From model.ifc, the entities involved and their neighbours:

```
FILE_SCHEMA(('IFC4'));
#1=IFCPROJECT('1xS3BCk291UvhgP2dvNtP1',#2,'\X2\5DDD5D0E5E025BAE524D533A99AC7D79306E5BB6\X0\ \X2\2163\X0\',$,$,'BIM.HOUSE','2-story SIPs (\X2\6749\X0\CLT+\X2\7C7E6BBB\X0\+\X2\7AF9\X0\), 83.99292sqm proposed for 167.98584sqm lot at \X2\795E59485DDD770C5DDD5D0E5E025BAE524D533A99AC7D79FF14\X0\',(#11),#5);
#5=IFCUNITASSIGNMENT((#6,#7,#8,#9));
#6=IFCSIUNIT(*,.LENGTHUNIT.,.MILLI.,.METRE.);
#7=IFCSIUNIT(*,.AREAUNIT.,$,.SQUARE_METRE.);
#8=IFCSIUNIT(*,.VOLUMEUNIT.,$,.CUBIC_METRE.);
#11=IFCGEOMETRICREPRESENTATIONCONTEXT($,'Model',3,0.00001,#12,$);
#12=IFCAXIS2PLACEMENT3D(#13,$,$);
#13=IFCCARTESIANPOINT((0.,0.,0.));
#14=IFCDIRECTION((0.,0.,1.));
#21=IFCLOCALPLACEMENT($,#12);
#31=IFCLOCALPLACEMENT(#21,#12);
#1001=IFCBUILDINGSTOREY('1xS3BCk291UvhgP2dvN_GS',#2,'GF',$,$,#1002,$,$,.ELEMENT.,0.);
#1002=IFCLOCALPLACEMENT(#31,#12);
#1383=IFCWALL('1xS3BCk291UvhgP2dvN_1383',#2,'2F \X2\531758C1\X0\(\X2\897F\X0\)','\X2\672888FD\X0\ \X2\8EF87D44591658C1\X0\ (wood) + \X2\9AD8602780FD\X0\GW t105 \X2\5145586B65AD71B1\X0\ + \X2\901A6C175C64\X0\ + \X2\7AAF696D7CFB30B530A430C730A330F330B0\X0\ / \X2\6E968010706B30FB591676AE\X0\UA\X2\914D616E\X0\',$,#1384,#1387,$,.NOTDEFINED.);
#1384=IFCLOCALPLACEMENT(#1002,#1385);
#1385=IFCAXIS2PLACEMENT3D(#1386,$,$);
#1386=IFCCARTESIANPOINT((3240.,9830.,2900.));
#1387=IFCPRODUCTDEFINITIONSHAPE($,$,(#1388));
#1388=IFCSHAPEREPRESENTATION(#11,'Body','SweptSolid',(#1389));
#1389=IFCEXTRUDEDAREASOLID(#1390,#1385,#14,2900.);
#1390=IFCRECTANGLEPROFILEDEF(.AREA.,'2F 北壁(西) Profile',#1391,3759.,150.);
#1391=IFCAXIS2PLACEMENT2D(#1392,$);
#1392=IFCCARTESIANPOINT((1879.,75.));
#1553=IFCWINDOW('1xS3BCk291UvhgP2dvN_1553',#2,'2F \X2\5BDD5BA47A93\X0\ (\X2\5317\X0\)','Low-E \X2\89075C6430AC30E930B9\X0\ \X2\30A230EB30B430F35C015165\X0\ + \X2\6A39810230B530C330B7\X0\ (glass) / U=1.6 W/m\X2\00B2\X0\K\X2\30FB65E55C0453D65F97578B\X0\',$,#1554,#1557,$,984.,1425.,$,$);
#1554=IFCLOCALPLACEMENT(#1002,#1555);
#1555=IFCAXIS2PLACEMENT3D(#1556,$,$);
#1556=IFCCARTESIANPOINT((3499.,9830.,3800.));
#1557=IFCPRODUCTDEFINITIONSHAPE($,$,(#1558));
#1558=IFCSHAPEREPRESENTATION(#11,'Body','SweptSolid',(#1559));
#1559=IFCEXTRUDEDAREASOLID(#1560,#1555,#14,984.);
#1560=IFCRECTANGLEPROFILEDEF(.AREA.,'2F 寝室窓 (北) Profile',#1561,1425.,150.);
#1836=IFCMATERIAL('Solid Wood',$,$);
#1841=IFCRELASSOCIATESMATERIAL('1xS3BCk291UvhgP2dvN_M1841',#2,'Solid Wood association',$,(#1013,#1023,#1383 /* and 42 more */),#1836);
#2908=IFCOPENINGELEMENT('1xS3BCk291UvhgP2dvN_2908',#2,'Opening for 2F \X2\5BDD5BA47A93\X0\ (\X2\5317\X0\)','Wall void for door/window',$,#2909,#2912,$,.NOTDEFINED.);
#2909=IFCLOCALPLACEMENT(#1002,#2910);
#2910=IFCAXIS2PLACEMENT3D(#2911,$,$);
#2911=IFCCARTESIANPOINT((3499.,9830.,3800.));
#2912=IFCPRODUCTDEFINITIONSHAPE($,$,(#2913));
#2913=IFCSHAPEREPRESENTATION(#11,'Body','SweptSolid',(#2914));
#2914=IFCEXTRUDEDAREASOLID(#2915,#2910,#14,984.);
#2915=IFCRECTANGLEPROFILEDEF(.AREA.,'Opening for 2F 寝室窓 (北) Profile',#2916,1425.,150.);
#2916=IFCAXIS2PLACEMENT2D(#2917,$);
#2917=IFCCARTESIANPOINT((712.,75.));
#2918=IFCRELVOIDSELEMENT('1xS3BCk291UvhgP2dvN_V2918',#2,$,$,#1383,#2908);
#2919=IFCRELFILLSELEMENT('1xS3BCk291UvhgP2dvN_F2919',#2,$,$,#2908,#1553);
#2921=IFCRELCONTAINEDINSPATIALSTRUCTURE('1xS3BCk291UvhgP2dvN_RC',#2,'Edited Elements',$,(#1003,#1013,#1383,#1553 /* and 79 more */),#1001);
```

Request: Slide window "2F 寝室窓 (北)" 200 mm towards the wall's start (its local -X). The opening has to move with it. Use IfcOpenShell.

```python
import ifcopenshell
import ifcopenshell.api.geometry
import ifcopenshell.util.placement

model = ifcopenshell.open("model.ifc")

window = model.by_id(1553)
opening = window.FillsVoids[0].RelatingOpeningElement
wall = opening.VoidsElements[0].RelatingBuildingElement

wall_matrix = ifcopenshell.util.placement.get_local_placement(wall.ObjectPlacement)
shift = wall_matrix[:3, 0] * -200.0
before = ifcopenshell.util.placement.get_local_placement(window.ObjectPlacement)[:3, 3].copy()

# The window is not placed relative to its opening, so move both.
for product in (opening, window):
    matrix = ifcopenshell.util.placement.get_local_placement(product.ObjectPlacement)
    matrix[:3, 3] += shift
    ifcopenshell.api.geometry.edit_object_placement(model, product=product, matrix=matrix, is_si=False)

after = ifcopenshell.util.placement.get_local_placement(window.ObjectPlacement)[:3, 3]
print("window moved by", (after - before).round(3) + 0.0)

model.write("model_rev.ifc")
```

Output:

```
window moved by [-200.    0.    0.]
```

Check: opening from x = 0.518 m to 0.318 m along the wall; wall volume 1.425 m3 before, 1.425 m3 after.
